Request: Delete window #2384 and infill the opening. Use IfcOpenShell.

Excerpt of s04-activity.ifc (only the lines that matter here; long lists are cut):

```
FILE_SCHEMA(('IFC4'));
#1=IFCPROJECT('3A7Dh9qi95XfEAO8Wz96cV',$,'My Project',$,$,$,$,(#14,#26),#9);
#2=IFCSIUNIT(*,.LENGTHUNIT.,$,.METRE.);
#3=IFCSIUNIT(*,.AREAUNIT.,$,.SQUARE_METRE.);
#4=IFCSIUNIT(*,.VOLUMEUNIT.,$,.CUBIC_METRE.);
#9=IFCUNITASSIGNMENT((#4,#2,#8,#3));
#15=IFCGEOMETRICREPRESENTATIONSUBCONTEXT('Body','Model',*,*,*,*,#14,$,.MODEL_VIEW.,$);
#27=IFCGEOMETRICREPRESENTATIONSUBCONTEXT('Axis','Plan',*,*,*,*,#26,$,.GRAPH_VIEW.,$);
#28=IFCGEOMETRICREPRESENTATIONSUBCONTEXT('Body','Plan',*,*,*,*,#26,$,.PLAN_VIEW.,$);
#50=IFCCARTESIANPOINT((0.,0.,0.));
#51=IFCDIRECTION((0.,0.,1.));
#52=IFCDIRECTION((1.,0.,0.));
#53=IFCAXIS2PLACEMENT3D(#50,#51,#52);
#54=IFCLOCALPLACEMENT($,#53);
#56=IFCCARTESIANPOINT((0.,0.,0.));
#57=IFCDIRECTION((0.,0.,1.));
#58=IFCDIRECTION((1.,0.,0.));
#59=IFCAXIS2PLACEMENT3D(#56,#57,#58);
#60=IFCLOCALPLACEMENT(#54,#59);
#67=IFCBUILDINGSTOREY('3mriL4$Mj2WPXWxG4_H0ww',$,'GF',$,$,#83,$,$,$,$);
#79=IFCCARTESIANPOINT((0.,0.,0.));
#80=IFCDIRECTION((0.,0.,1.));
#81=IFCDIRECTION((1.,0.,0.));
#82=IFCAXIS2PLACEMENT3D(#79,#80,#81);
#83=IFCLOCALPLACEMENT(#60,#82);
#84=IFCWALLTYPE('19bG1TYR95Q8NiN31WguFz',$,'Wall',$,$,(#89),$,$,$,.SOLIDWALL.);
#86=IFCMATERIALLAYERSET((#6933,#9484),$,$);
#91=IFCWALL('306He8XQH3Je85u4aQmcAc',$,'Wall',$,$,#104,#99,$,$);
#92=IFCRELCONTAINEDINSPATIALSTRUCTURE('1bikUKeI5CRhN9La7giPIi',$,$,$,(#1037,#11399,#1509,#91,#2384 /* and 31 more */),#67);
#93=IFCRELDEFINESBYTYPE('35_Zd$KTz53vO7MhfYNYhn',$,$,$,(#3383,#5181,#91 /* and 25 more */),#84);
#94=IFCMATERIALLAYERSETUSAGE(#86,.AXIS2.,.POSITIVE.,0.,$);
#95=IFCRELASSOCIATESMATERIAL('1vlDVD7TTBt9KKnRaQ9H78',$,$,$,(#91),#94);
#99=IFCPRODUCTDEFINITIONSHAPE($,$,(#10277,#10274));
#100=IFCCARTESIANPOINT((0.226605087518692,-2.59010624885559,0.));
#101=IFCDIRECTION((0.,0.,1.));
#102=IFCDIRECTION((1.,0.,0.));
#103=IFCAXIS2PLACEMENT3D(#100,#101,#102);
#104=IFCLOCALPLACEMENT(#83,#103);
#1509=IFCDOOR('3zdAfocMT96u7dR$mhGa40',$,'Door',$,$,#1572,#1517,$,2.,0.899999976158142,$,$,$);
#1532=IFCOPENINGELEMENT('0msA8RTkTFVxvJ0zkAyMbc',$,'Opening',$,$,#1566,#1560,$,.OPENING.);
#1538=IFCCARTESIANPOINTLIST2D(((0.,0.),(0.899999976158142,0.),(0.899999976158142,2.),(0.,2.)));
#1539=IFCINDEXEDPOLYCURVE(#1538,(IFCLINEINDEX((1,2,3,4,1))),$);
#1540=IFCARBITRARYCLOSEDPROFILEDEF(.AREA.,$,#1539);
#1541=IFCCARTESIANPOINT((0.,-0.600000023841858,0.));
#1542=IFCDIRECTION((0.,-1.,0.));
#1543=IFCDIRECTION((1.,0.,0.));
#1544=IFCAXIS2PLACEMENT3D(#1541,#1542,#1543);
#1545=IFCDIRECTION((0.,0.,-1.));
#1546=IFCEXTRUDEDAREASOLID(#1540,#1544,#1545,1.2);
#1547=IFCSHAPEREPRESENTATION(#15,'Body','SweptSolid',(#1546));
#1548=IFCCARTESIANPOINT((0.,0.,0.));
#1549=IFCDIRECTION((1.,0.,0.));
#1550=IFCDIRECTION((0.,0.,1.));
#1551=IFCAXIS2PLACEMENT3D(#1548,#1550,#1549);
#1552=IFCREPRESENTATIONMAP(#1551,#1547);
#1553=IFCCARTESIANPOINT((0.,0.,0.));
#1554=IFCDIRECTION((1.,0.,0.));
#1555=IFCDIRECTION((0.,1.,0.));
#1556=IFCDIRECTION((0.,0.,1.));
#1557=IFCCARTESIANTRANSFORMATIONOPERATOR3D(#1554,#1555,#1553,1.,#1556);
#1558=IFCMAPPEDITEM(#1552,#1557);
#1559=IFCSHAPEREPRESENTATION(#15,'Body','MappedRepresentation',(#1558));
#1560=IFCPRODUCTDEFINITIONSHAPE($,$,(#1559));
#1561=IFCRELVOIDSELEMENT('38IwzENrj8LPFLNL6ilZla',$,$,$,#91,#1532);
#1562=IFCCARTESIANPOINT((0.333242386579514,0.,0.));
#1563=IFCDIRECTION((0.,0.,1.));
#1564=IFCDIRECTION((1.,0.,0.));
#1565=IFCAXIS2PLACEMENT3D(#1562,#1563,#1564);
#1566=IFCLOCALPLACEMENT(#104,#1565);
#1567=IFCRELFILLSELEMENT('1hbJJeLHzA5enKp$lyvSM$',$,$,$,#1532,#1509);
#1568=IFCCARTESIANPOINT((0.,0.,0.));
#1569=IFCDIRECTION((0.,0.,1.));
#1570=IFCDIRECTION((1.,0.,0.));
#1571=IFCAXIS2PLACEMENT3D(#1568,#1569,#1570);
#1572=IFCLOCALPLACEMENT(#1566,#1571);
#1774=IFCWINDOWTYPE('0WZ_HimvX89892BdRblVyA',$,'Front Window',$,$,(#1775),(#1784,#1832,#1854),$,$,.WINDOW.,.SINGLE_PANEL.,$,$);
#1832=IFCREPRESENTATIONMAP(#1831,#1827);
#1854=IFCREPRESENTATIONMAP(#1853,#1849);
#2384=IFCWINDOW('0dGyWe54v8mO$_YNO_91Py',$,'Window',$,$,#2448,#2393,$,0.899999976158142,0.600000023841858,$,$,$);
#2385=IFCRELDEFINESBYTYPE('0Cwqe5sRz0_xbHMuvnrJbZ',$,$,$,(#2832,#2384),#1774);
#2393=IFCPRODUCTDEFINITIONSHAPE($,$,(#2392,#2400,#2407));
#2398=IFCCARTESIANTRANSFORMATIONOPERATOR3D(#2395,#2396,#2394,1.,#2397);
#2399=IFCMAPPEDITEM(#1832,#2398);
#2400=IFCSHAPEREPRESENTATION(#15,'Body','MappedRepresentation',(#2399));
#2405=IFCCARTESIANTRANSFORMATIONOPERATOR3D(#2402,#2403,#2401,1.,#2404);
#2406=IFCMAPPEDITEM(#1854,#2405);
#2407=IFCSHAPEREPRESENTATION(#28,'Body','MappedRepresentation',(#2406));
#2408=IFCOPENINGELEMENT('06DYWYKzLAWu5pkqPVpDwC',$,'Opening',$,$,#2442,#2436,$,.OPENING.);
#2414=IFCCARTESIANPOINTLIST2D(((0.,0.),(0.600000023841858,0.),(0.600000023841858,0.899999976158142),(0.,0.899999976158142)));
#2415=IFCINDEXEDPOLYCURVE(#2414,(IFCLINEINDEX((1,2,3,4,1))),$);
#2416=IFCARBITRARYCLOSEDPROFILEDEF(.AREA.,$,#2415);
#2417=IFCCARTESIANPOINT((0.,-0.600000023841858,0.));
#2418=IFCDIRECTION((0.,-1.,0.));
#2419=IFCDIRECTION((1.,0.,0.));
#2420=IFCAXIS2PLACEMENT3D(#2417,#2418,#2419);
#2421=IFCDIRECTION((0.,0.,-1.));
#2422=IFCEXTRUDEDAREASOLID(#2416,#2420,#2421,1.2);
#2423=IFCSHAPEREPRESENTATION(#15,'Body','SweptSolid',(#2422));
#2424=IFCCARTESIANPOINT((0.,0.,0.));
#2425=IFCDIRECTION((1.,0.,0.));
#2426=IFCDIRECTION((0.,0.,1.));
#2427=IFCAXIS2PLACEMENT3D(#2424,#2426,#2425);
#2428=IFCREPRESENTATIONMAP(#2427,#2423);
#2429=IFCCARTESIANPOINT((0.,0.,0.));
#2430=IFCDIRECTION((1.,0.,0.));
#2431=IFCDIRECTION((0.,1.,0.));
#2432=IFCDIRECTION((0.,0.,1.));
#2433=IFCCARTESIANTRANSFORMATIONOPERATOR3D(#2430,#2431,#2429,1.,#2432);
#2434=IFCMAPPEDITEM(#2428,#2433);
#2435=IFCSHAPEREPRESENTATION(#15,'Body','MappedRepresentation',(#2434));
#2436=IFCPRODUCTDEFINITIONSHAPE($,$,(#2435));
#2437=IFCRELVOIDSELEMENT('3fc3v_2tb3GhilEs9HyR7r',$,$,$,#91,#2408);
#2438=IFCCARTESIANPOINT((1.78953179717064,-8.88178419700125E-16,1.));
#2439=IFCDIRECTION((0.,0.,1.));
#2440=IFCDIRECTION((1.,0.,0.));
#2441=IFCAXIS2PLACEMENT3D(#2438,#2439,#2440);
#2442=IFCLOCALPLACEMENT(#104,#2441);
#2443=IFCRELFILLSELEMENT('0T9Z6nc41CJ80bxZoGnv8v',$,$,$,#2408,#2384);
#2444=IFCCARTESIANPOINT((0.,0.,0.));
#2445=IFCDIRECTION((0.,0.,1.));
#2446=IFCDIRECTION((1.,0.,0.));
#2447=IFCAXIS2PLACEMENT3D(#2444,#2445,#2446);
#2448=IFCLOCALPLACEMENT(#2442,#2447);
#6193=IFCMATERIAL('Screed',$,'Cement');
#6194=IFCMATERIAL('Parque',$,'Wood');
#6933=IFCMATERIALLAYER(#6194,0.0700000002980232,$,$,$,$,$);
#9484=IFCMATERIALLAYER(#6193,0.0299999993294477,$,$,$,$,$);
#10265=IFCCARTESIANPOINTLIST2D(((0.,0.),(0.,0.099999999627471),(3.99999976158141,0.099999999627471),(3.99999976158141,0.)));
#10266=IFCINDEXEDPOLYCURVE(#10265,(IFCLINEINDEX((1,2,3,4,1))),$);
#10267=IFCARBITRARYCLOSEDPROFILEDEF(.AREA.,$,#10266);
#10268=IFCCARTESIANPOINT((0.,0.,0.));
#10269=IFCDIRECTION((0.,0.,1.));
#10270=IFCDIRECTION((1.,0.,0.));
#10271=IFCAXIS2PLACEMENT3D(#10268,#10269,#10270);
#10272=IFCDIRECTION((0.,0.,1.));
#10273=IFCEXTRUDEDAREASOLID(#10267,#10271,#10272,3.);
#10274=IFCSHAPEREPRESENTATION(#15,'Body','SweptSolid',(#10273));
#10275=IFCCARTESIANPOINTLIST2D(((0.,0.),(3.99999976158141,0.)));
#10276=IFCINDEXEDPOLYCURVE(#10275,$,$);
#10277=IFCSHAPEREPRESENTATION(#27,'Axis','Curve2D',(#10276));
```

```python
import ifcopenshell
import ifcopenshell.api.feature
import ifcopenshell.api.root
import ifcopenshell.geom
import ifcopenshell.util.shape

model = ifcopenshell.open("s04-activity.ifc")
settings = ifcopenshell.geom.settings()


def volume(element):
    """Net volume in cubic metres, openings subtracted."""
    shape = ifcopenshell.geom.create_shape(settings, element)
    return ifcopenshell.util.shape.get_volume(shape.geometry)


window = model.by_guid("0dGyWe54v8mO$_YNO_91Py")
opening = window.FillsVoids[0].RelatingOpeningElement
wall = opening.VoidsElements[0].RelatingBuildingElement
before = volume(wall)

ifcopenshell.api.root.remove_product(model, product=window)
ifcopenshell.api.feature.remove_feature(model, feature=opening)

after = volume(wall)

print(f"wall volume {before:.3f} -> {after:.3f} m3")

model.write("s04-activity-out.ifc")
```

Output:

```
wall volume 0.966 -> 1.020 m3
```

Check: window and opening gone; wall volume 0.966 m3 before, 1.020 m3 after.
